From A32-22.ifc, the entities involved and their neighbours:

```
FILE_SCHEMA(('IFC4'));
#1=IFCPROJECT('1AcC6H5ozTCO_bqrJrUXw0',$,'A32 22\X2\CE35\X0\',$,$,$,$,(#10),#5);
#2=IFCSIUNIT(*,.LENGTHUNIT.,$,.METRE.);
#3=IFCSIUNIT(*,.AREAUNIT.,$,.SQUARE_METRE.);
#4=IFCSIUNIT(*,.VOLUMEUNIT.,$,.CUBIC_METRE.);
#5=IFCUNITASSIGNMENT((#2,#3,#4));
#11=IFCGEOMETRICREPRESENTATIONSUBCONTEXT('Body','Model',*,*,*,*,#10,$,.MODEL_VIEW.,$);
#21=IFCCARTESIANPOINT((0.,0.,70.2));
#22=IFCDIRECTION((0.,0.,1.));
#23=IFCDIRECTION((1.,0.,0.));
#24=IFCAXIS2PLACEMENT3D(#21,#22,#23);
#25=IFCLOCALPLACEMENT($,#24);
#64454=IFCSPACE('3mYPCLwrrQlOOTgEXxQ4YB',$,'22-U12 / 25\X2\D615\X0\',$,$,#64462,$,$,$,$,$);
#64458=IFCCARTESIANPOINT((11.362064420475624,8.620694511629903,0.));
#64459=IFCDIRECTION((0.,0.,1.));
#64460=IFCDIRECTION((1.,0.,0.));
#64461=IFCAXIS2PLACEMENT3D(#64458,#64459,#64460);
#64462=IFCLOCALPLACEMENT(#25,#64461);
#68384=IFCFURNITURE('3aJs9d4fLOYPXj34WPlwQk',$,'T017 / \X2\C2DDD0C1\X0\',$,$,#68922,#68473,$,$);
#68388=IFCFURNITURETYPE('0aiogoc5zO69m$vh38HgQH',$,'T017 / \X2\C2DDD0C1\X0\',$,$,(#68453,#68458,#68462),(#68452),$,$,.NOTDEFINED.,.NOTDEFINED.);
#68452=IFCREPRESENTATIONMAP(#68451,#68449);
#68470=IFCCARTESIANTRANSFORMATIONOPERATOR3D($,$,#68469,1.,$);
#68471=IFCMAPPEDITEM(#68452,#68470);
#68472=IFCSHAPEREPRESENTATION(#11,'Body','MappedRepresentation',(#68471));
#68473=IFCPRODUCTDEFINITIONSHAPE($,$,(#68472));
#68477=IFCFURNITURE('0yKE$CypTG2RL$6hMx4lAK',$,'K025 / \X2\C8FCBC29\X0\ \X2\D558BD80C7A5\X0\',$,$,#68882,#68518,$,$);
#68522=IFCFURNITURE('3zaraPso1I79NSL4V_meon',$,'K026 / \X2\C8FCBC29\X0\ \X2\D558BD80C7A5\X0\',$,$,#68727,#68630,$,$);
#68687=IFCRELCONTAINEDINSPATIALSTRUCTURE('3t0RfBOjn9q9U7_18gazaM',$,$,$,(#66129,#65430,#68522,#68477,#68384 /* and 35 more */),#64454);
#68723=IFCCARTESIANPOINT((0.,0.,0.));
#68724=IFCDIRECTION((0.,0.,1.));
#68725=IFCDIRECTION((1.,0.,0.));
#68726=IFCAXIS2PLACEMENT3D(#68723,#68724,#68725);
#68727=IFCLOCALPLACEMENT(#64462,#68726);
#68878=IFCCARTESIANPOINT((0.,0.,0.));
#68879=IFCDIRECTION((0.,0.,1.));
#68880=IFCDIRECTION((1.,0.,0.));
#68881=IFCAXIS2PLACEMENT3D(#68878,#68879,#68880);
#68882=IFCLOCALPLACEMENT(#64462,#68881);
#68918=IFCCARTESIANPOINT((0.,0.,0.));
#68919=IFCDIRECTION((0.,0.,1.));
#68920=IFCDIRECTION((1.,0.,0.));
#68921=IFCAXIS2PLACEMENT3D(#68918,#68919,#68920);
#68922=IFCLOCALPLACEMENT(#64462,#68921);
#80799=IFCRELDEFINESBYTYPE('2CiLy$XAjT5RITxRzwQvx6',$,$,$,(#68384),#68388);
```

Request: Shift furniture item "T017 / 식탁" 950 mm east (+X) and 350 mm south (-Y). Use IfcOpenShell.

```python
import ifcopenshell
import ifcopenshell.api.geometry
import ifcopenshell.util.placement
import ifcopenshell.util.unit

model = ifcopenshell.open("A32-22.ifc")
unit_scale = ifcopenshell.util.unit.calculate_unit_scale(model)

item = model.by_guid("3aJs9d4fLOYPXj34WPlwQk")
matrix = ifcopenshell.util.placement.get_local_placement(item.ObjectPlacement)
matrix[0, 3] += 0.95 / unit_scale
matrix[1, 3] -= 0.35 / unit_scale
ifcopenshell.api.geometry.edit_object_placement(model, product=item, matrix=matrix, is_si=False)

print(ifcopenshell.util.placement.get_local_placement(item.ObjectPlacement).round(3) + 0.0)

model.write("A32-22_v2.ifc")
```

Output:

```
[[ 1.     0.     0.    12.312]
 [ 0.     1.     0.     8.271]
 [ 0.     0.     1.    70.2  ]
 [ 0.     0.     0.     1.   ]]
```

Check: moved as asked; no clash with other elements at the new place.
